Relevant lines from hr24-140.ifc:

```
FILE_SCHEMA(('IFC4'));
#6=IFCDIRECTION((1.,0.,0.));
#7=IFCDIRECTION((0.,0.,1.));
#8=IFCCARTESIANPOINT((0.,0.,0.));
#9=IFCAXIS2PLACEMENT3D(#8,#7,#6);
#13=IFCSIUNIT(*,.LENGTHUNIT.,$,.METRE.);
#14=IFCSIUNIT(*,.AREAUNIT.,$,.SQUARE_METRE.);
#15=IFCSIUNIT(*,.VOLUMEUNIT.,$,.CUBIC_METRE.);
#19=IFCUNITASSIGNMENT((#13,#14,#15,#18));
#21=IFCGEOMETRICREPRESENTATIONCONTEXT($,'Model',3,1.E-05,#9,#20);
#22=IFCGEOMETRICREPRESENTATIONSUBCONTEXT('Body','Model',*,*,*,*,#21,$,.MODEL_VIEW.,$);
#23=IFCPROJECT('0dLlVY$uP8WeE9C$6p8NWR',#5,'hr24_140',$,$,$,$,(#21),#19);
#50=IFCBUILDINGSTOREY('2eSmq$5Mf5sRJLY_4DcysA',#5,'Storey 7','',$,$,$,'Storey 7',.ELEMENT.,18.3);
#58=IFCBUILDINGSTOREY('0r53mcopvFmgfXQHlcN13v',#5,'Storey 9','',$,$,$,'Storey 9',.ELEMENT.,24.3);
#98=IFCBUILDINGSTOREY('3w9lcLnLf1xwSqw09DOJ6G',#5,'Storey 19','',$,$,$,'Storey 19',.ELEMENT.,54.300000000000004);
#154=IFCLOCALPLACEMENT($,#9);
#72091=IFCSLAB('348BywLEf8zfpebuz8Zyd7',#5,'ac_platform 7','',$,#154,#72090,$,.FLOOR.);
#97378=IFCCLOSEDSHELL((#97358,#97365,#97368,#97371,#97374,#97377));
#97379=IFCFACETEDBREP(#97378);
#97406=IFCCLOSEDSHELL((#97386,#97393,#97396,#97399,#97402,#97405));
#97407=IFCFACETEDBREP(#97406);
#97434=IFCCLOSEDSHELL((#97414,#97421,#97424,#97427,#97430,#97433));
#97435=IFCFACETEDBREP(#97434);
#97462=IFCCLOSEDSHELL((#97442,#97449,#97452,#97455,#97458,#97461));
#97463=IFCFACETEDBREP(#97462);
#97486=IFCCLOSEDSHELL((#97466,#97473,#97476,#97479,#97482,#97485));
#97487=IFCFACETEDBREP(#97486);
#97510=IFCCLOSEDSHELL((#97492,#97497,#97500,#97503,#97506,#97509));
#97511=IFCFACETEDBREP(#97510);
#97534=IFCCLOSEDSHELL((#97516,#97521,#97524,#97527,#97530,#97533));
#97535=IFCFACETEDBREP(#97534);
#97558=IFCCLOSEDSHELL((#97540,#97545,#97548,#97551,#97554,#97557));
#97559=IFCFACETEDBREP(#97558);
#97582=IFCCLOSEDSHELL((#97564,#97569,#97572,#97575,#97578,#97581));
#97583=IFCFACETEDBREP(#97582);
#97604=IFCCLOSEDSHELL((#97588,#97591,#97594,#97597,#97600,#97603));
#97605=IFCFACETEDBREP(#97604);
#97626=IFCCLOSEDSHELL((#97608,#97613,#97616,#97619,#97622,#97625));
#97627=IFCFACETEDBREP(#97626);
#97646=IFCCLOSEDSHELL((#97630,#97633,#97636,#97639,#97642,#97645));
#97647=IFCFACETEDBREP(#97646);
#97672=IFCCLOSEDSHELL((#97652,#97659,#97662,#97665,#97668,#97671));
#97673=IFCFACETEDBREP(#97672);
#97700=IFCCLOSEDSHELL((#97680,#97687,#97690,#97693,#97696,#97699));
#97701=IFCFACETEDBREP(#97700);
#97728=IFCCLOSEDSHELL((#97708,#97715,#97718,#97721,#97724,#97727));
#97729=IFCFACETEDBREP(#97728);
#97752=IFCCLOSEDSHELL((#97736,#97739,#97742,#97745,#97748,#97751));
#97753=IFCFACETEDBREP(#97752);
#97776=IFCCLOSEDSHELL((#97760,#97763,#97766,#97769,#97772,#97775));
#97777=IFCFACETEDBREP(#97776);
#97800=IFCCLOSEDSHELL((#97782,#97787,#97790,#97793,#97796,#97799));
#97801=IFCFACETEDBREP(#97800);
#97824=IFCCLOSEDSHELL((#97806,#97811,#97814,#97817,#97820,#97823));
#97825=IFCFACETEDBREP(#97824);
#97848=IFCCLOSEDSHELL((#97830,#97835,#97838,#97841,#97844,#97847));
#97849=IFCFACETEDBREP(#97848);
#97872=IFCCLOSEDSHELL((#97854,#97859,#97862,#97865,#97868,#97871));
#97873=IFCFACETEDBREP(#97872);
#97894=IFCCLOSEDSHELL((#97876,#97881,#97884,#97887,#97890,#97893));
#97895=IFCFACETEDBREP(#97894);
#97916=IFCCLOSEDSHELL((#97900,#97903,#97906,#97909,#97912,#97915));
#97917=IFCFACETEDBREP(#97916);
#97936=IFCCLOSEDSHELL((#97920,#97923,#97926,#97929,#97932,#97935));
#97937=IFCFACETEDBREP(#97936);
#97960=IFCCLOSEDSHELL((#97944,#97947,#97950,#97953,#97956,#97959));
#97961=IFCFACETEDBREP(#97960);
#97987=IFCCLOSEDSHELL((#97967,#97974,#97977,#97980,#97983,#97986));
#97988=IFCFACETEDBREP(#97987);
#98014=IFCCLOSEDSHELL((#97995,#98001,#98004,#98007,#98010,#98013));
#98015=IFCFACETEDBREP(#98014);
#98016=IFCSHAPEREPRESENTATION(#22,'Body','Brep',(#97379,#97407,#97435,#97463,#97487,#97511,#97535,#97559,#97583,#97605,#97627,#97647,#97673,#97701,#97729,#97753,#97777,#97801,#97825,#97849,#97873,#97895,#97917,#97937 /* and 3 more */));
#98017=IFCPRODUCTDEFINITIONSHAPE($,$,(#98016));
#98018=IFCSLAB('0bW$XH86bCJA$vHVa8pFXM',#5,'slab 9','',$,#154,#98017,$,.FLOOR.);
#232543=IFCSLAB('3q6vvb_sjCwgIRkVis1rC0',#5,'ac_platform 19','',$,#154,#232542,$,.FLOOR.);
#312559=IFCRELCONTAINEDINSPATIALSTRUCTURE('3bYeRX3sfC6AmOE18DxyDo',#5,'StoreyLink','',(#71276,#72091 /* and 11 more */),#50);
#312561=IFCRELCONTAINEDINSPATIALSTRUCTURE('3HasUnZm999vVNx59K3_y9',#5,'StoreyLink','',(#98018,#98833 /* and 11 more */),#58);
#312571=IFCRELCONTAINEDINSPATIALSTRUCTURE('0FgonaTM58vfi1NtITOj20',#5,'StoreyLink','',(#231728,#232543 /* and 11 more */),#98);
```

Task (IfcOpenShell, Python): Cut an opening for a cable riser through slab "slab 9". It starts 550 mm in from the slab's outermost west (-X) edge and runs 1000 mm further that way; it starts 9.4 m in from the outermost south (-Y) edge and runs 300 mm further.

```python
import numpy as np
import ifcopenshell
import ifcopenshell.api.feature
import ifcopenshell.api.geometry
import ifcopenshell.api.root
import ifcopenshell.geom
import ifcopenshell.util.placement
import ifcopenshell.util.representation
import ifcopenshell.util.shape
import ifcopenshell.util.unit

model = ifcopenshell.open("hr24-140.ifc")
unit_scale = ifcopenshell.util.unit.calculate_unit_scale(model)
settings = ifcopenshell.geom.settings()


def volume(element):
    """Net volume in cubic metres, openings subtracted."""
    shape = ifcopenshell.geom.create_shape(settings, element)
    return ifcopenshell.util.shape.get_volume(shape.geometry)


slab = model.by_id(98018)
before = volume(slab)

# Extent in the slab's own axes, in metres. The edges named are its -X and -Y sides.
slab_shape = ifcopenshell.geom.create_shape(settings, slab)
vertices = ifcopenshell.util.shape.get_vertices(slab_shape.geometry)
x_min, y_min, bottom = vertices.min(axis=0)
top = vertices[:, 2].max()

opening = ifcopenshell.api.root.create_entity(model, ifc_class="IfcOpeningElement", name="Cable riser opening", predefined_type="OPENING")
context = ifcopenshell.util.representation.get_context(model, "Model", "Body", "MODEL_VIEW")
width, depth = 1, 0.3
outline = [(0.0, 0.0), (width, 0.0), (width, depth), (0.0, depth), (0.0, 0.0)]
# Overshoot both faces by 50 mm so the cut is clean.
shape = ifcopenshell.api.geometry.add_slab_representation(
    model, context=context, depth=top - bottom + 0.1, polyline=outline
)
ifcopenshell.api.geometry.assign_representation(model, product=opening, representation=shape)

matrix = ifcopenshell.util.placement.get_local_placement(slab.ObjectPlacement)
matrix[:, 3] = matrix @ np.append(np.array([x_min + 0.55, y_min + 9.4, bottom - 0.05]) / unit_scale, 1.0)
ifcopenshell.api.geometry.edit_object_placement(model, product=opening, matrix=matrix, is_si=False)
ifcopenshell.api.feature.add_feature(model, feature=opening, element=slab)

after = volume(slab)

print(f"slab volume {before:.3f} -> {after:.3f} m3")

model.write("hr24-140_v2.ifc")
```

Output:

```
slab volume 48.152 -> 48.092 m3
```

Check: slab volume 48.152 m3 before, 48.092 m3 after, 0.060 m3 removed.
